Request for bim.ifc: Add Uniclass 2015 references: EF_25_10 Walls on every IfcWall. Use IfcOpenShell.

First a look at what the model holds.

```python
import ifcopenshell

model = ifcopenshell.open("bim.ifc")
print(model.schema)
print("classifications:", [c.Name for c in model.by_type("IfcClassification")])
for ifc_class in ("IfcDoor", "IfcRoof", "IfcStair", "IfcWall", "IfcWindow"):
    print(ifc_class, len(model.by_type(ifc_class)))
```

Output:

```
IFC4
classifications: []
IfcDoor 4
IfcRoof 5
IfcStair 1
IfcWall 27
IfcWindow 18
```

```python
import ifcopenshell
import ifcopenshell.api.classification

model = ifcopenshell.open("bim.ifc")

system = ifcopenshell.api.classification.add_classification(model, classification="Uniclass 2015")

codes = {
    "IfcWall": ("EF_25_10", "Walls"),
}
for ifc_class, (code, name) in codes.items():
    products = model.by_type(ifc_class)
    ifcopenshell.api.classification.add_reference(
        model, products=products, classification=system, identification=code, name=name
    )
    print(code, len(products))

model.write("bim_edited.ifc")
```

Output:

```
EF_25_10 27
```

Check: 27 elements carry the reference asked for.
